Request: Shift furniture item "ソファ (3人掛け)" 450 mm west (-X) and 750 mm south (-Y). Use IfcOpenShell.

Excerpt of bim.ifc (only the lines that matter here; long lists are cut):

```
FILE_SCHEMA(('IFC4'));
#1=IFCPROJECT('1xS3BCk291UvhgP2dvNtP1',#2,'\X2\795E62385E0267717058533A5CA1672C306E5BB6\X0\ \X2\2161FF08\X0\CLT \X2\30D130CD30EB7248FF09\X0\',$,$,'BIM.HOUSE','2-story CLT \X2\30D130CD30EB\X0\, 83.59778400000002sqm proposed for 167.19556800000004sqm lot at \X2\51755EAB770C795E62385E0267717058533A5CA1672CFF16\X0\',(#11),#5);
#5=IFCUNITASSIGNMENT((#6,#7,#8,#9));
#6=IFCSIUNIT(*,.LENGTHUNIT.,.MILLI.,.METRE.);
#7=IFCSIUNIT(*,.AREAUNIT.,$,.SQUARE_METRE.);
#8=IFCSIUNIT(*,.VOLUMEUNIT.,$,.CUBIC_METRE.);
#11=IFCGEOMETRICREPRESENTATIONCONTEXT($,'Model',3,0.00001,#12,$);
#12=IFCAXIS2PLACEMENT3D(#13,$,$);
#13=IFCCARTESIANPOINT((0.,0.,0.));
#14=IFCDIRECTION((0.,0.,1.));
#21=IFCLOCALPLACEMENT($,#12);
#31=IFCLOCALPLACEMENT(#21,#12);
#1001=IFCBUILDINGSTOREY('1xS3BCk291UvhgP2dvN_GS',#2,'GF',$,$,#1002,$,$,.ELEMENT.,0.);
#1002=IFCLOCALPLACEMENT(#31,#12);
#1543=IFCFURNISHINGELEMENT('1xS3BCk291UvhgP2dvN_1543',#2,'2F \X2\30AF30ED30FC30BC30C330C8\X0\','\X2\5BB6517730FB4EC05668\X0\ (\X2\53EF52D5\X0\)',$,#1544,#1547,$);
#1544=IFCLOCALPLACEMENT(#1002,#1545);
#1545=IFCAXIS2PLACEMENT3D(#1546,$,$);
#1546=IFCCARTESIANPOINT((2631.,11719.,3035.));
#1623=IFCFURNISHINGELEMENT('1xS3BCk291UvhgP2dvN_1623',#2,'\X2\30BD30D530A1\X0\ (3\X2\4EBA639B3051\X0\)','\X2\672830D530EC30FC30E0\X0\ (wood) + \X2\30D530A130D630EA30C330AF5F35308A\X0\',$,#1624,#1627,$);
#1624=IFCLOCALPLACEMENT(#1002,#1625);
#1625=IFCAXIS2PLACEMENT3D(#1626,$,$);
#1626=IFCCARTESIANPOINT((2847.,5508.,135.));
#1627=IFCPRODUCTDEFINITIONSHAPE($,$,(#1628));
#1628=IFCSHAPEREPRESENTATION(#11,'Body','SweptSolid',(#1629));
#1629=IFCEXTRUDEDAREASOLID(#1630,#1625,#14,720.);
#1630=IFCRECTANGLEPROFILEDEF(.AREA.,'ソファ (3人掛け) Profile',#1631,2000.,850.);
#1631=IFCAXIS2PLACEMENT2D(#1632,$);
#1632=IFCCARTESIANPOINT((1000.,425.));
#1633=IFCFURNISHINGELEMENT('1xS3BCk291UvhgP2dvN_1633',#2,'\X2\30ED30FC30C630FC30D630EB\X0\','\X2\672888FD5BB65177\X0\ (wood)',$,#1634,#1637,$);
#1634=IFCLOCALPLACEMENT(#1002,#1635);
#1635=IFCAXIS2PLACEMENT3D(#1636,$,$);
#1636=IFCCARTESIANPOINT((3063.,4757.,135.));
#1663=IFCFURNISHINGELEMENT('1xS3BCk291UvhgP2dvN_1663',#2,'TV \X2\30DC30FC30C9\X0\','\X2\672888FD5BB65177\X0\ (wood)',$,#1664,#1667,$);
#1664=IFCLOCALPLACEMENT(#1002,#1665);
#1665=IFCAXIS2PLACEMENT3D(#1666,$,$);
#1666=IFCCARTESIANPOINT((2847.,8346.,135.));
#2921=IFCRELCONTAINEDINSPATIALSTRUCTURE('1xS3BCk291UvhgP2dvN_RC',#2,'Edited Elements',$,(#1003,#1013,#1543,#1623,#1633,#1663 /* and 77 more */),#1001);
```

```python
import ifcopenshell
import ifcopenshell.api.geometry
import ifcopenshell.util.placement
import ifcopenshell.util.unit

model = ifcopenshell.open("bim.ifc")
unit_scale = ifcopenshell.util.unit.calculate_unit_scale(model)

item = model.by_guid("1xS3BCk291UvhgP2dvN_1623")
matrix = ifcopenshell.util.placement.get_local_placement(item.ObjectPlacement)
matrix[0, 3] -= 0.45 / unit_scale
matrix[1, 3] -= 0.75 / unit_scale
ifcopenshell.api.geometry.edit_object_placement(model, product=item, matrix=matrix, is_si=False)

print(ifcopenshell.util.placement.get_local_placement(item.ObjectPlacement).round(3) + 0.0)

model.write("bim_updated.ifc")
```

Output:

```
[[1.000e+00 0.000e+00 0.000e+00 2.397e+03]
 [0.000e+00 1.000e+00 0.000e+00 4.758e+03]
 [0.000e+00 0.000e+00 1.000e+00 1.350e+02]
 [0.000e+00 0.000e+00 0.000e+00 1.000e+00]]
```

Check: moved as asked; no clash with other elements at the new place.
